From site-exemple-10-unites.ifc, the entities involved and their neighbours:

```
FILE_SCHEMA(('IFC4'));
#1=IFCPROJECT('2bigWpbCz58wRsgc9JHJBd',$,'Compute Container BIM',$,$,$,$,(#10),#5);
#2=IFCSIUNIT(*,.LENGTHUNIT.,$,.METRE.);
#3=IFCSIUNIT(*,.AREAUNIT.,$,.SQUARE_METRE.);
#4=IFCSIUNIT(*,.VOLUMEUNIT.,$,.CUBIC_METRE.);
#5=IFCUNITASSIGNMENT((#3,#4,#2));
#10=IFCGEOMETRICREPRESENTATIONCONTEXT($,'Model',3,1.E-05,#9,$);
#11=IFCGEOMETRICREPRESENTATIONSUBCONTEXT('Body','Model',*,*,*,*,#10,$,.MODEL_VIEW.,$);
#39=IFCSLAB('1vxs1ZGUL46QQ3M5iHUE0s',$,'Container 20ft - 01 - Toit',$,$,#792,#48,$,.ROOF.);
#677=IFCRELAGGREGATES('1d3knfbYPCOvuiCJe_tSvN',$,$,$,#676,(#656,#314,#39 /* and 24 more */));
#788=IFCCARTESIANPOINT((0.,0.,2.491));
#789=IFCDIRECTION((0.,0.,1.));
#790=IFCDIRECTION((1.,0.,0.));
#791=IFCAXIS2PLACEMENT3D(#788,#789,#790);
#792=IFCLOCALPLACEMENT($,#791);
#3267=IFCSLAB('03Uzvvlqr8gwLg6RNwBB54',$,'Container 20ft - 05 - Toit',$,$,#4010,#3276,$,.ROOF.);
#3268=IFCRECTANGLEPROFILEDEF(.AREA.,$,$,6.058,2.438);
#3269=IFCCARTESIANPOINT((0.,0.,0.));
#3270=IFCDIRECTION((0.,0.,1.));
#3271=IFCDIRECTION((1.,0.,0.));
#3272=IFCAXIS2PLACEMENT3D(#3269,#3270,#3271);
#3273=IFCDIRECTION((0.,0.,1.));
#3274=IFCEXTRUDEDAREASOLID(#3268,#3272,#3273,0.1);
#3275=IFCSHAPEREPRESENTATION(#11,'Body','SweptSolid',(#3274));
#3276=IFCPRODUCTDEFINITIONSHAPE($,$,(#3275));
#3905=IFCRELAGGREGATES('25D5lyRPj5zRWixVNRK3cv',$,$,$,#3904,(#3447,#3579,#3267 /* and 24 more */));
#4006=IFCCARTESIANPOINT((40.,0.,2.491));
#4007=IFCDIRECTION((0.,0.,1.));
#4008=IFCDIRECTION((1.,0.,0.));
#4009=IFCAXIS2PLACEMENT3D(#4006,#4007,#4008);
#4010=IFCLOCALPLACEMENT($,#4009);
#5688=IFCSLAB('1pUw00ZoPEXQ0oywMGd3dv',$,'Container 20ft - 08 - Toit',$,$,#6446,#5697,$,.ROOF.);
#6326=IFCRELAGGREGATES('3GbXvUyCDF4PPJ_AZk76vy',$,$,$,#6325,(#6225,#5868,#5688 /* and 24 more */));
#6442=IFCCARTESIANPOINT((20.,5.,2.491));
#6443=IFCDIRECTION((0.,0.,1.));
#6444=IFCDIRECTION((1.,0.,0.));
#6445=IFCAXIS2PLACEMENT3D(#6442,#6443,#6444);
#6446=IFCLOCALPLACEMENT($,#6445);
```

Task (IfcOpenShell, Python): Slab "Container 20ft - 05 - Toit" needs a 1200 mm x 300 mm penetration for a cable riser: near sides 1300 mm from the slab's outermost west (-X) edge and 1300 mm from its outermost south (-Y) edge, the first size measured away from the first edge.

```python
import numpy as np
import ifcopenshell
import ifcopenshell.api.feature
import ifcopenshell.api.geometry
import ifcopenshell.api.root
import ifcopenshell.geom
import ifcopenshell.util.placement
import ifcopenshell.util.representation
import ifcopenshell.util.shape
import ifcopenshell.util.unit

model = ifcopenshell.open("site-exemple-10-unites.ifc")
unit_scale = ifcopenshell.util.unit.calculate_unit_scale(model)
settings = ifcopenshell.geom.settings()


def volume(element):
    """Net volume in cubic metres, openings subtracted."""
    shape = ifcopenshell.geom.create_shape(settings, element)
    return ifcopenshell.util.shape.get_volume(shape.geometry)


slab = model.by_id(3267)
before = volume(slab)

# Extent in the slab's own axes, in metres. The edges named are its -X and -Y sides.
slab_shape = ifcopenshell.geom.create_shape(settings, slab)
vertices = ifcopenshell.util.shape.get_vertices(slab_shape.geometry)
x_min, y_min, bottom = vertices.min(axis=0)
top = vertices[:, 2].max()

opening = ifcopenshell.api.root.create_entity(model, ifc_class="IfcOpeningElement", name="Cable riser opening", predefined_type="OPENING")
context = ifcopenshell.util.representation.get_context(model, "Model", "Body", "MODEL_VIEW")
width, depth = 1.2, 0.3
outline = [(0.0, 0.0), (width, 0.0), (width, depth), (0.0, depth), (0.0, 0.0)]
# Overshoot both faces by 50 mm so the cut is clean.
shape = ifcopenshell.api.geometry.add_slab_representation(
    model, context=context, depth=top - bottom + 0.1, polyline=outline
)
ifcopenshell.api.geometry.assign_representation(model, product=opening, representation=shape)

matrix = ifcopenshell.util.placement.get_local_placement(slab.ObjectPlacement)
matrix[:, 3] = matrix @ np.append(np.array([x_min + 1.3, y_min + 1.3, bottom - 0.05]) / unit_scale, 1.0)
ifcopenshell.api.geometry.edit_object_placement(model, product=opening, matrix=matrix, is_si=False)
ifcopenshell.api.feature.add_feature(model, feature=opening, element=slab)

after = volume(slab)

print(f"slab volume {before:.3f} -> {after:.3f} m3")

model.write("site-exemple-10-unites_updated.ifc")
```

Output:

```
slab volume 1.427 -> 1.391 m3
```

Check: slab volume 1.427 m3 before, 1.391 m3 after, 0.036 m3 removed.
